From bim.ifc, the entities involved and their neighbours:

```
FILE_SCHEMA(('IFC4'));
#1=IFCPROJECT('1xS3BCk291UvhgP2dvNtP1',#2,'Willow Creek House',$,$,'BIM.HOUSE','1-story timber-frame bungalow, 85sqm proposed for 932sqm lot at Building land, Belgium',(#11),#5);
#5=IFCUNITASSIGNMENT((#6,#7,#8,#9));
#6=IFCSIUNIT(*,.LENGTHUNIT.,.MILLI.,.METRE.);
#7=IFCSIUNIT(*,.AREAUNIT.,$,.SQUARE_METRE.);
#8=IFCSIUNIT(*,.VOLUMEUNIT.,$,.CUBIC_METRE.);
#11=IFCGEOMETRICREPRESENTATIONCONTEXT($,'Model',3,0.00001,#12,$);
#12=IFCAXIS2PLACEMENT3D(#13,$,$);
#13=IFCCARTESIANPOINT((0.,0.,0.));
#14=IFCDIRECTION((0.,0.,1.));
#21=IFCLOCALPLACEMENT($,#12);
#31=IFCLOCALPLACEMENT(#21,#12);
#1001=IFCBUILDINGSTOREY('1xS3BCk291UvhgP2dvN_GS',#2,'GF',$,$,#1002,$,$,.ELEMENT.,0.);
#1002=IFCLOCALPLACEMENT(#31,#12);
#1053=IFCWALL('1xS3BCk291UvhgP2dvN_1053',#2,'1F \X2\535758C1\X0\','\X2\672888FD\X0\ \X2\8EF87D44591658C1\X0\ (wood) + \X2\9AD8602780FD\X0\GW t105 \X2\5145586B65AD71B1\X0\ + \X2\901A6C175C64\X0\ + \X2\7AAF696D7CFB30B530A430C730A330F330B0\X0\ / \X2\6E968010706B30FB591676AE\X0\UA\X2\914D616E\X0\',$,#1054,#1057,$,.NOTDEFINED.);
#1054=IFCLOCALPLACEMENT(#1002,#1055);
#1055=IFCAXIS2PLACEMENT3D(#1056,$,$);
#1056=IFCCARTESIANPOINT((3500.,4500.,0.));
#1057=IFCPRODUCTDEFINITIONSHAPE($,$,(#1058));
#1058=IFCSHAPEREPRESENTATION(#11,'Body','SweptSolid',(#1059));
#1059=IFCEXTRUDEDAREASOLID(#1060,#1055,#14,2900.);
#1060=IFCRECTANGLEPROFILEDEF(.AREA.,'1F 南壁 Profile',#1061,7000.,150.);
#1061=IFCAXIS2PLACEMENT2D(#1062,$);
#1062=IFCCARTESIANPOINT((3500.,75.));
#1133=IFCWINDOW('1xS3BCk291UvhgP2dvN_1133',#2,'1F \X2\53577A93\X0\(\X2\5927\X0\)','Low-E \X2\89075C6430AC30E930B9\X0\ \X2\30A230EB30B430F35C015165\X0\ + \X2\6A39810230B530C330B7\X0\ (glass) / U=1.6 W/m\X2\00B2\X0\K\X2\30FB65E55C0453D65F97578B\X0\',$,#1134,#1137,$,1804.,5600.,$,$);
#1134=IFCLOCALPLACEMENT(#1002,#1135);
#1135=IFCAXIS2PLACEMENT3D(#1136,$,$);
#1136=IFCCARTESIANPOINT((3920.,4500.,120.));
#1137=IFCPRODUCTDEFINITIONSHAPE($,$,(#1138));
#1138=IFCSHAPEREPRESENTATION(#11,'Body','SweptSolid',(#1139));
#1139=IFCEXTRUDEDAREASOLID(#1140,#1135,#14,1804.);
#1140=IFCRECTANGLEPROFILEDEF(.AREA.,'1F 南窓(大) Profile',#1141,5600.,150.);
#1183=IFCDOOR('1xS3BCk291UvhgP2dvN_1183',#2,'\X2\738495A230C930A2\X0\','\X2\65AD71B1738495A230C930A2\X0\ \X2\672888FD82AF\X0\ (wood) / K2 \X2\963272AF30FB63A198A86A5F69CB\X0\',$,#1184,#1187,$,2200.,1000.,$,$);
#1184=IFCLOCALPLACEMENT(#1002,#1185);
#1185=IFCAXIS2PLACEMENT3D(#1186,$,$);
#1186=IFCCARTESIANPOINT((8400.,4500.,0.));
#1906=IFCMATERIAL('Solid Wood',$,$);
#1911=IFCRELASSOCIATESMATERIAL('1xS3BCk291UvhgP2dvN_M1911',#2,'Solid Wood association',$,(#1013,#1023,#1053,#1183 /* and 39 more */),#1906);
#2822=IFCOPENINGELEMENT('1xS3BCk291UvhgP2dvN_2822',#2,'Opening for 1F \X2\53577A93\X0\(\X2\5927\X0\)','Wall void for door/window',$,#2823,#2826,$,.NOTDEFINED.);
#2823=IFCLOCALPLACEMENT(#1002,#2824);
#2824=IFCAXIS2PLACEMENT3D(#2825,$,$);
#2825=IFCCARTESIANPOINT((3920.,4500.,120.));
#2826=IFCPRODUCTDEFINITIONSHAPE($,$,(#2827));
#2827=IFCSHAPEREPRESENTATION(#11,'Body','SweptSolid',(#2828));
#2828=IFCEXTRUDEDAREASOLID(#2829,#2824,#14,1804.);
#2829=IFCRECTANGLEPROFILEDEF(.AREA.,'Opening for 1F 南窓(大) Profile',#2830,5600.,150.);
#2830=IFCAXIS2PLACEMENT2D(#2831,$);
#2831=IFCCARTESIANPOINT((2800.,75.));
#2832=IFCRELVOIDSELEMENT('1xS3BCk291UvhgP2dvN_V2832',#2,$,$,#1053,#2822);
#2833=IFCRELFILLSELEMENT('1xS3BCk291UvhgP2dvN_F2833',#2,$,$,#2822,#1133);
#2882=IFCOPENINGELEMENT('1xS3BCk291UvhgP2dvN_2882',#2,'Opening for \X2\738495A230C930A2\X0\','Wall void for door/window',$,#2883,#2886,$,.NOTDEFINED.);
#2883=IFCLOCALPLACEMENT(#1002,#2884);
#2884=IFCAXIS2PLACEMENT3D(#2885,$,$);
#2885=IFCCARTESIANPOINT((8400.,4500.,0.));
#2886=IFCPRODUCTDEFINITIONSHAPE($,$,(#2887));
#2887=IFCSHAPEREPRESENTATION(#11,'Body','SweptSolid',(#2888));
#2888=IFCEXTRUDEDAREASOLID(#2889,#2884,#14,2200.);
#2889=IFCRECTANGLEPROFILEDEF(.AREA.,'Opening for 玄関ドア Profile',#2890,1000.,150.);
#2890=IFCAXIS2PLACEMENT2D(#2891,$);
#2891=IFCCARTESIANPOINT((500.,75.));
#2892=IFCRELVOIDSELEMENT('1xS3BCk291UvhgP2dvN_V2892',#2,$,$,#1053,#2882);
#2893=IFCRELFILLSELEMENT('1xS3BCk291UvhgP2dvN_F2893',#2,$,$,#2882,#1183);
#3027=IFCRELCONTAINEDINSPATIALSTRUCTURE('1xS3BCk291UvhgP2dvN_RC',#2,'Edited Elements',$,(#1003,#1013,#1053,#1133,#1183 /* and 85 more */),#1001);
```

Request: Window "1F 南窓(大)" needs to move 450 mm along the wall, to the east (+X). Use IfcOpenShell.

```python
import ifcopenshell
import ifcopenshell.api.geometry
import ifcopenshell.util.placement
import ifcopenshell.util.unit

model = ifcopenshell.open("bim.ifc")
unit_scale = ifcopenshell.util.unit.calculate_unit_scale(model)

window = model.by_id(1133)
opening = window.FillsVoids[0].RelatingOpeningElement
wall = opening.VoidsElements[0].RelatingBuildingElement

wall_matrix = ifcopenshell.util.placement.get_local_placement(wall.ObjectPlacement)
shift = wall_matrix[:3, 0] * 0.45 / unit_scale
before = ifcopenshell.util.placement.get_local_placement(window.ObjectPlacement)[:3, 3].copy()

# The window is not placed relative to its opening, so move both.
for product in (opening, window):
    matrix = ifcopenshell.util.placement.get_local_placement(product.ObjectPlacement)
    matrix[:3, 3] += shift
    ifcopenshell.api.geometry.edit_object_placement(model, product=product, matrix=matrix, is_si=False)

after = ifcopenshell.util.placement.get_local_placement(window.ObjectPlacement)[:3, 3]
print("window moved by", (after - before).round(3) + 0.0)

model.write("bim_rev.ifc")
```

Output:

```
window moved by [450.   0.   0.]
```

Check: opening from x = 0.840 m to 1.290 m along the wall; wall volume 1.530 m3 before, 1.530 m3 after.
